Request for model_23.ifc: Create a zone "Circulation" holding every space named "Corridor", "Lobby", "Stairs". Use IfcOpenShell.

First a look at what the model holds.

```python
import ifcopenshell

model = ifcopenshell.open("model_23.ifc")
print(model.schema)
seen = {}
for space in model.by_type("IfcSpace"):
    seen[space.LongName] = seen.get(space.LongName, 0) + 1
for name, count in sorted(seen.items(), key=str):
    print(count, "x", name)
print("zones:", [z.Name for z in model.by_type("IfcZone")][:20])
```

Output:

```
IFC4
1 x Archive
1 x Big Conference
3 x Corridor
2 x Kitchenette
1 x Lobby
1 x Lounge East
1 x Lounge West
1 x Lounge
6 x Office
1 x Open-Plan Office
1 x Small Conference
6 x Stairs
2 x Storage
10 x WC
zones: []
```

```python
import ifcopenshell
import ifcopenshell.api.group
import ifcopenshell.api.root

model = ifcopenshell.open("model_23.ifc")

names = {"Corridor", "Lobby", "Stairs"}
spaces = [s for s in model.by_type("IfcSpace") if s.LongName in names]

zone = ifcopenshell.api.root.create_entity(model, ifc_class="IfcZone", name="Circulation")
ifcopenshell.api.group.assign_group(model, products=spaces, group=zone)
print(len(spaces), "spaces in", zone.Name)

model.write("model_23_edited.ifc")
```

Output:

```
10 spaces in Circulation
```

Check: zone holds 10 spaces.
